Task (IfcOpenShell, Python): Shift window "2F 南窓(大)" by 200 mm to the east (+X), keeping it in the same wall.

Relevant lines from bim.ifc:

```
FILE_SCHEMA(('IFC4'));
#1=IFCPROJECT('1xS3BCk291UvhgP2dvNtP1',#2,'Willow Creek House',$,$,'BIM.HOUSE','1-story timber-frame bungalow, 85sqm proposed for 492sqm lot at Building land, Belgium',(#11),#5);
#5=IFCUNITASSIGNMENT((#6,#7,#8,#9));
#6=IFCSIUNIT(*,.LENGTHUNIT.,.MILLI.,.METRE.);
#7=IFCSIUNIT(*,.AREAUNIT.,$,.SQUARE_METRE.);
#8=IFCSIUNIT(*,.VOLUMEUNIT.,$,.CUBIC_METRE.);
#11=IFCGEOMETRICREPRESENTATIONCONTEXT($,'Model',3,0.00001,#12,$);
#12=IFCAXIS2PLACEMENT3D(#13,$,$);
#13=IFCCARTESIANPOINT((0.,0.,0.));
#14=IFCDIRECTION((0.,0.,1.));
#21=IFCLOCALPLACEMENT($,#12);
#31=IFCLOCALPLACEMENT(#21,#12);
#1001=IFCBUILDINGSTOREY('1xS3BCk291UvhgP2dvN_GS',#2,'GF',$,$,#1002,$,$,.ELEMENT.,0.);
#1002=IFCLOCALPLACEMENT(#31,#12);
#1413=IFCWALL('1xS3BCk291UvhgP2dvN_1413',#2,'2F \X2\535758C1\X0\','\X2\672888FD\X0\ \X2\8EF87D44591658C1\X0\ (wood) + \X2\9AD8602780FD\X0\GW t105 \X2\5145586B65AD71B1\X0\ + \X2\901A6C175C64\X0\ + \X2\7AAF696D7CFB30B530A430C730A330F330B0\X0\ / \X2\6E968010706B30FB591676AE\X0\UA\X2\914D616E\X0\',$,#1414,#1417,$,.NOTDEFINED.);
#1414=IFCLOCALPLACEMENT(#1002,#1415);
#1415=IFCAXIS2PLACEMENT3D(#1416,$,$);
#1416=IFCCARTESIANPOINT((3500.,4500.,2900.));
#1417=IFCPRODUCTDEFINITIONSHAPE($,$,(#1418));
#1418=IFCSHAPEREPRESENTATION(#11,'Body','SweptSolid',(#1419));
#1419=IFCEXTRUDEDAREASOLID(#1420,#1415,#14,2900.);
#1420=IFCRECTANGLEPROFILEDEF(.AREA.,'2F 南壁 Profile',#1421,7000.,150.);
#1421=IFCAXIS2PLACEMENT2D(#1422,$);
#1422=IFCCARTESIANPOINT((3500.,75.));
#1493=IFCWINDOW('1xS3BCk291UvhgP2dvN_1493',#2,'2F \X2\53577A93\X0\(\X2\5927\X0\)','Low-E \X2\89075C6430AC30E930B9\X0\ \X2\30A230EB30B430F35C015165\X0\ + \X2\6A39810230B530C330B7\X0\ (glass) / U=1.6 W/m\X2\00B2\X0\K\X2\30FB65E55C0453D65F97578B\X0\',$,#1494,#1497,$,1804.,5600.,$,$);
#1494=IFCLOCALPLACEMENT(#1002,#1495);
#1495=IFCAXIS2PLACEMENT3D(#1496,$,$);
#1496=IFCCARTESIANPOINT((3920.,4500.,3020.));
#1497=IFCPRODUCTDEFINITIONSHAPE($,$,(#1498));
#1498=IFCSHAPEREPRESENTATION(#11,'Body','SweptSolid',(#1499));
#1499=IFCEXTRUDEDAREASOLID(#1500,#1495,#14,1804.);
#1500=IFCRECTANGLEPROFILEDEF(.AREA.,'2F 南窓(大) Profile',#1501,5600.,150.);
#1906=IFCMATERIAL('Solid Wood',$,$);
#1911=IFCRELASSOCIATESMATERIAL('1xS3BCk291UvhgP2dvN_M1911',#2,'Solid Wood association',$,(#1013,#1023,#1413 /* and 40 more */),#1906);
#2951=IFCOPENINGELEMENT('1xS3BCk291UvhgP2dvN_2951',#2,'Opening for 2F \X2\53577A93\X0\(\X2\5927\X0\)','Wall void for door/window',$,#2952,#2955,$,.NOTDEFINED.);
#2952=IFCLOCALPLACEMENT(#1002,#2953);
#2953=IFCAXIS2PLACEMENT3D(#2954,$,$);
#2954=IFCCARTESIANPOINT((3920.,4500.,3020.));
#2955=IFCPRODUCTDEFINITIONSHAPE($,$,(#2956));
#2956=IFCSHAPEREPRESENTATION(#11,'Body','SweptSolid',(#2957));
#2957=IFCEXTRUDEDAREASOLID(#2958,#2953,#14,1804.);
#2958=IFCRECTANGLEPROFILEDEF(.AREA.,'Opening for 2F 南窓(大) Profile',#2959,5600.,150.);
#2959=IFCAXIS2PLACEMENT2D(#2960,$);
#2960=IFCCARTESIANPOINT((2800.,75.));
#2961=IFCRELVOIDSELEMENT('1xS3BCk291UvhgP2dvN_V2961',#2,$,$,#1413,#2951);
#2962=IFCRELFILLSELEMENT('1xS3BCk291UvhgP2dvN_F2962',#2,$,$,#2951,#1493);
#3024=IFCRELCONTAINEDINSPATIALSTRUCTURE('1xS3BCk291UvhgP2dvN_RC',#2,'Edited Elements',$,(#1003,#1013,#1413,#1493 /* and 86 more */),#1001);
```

```python
import ifcopenshell
import ifcopenshell.api.geometry
import ifcopenshell.util.placement

model = ifcopenshell.open("bim.ifc")

window = model.by_guid("1xS3BCk291UvhgP2dvN_1493")
opening = window.FillsVoids[0].RelatingOpeningElement
wall = opening.VoidsElements[0].RelatingBuildingElement

wall_matrix = ifcopenshell.util.placement.get_local_placement(wall.ObjectPlacement)
shift = wall_matrix[:3, 0] * 200.0
before = ifcopenshell.util.placement.get_local_placement(window.ObjectPlacement)[:3, 3].copy()

# The window is not placed relative to its opening, so move both.
for product in (opening, window):
    matrix = ifcopenshell.util.placement.get_local_placement(product.ObjectPlacement)
    matrix[:3, 3] += shift
    ifcopenshell.api.geometry.edit_object_placement(model, product=product, matrix=matrix, is_si=False)

after = ifcopenshell.util.placement.get_local_placement(window.ObjectPlacement)[:3, 3]
print("window moved by", (after - before).round(3) + 0.0)

model.write("bim_v2.ifc")
```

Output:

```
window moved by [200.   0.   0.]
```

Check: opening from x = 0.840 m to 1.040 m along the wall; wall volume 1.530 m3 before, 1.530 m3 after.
